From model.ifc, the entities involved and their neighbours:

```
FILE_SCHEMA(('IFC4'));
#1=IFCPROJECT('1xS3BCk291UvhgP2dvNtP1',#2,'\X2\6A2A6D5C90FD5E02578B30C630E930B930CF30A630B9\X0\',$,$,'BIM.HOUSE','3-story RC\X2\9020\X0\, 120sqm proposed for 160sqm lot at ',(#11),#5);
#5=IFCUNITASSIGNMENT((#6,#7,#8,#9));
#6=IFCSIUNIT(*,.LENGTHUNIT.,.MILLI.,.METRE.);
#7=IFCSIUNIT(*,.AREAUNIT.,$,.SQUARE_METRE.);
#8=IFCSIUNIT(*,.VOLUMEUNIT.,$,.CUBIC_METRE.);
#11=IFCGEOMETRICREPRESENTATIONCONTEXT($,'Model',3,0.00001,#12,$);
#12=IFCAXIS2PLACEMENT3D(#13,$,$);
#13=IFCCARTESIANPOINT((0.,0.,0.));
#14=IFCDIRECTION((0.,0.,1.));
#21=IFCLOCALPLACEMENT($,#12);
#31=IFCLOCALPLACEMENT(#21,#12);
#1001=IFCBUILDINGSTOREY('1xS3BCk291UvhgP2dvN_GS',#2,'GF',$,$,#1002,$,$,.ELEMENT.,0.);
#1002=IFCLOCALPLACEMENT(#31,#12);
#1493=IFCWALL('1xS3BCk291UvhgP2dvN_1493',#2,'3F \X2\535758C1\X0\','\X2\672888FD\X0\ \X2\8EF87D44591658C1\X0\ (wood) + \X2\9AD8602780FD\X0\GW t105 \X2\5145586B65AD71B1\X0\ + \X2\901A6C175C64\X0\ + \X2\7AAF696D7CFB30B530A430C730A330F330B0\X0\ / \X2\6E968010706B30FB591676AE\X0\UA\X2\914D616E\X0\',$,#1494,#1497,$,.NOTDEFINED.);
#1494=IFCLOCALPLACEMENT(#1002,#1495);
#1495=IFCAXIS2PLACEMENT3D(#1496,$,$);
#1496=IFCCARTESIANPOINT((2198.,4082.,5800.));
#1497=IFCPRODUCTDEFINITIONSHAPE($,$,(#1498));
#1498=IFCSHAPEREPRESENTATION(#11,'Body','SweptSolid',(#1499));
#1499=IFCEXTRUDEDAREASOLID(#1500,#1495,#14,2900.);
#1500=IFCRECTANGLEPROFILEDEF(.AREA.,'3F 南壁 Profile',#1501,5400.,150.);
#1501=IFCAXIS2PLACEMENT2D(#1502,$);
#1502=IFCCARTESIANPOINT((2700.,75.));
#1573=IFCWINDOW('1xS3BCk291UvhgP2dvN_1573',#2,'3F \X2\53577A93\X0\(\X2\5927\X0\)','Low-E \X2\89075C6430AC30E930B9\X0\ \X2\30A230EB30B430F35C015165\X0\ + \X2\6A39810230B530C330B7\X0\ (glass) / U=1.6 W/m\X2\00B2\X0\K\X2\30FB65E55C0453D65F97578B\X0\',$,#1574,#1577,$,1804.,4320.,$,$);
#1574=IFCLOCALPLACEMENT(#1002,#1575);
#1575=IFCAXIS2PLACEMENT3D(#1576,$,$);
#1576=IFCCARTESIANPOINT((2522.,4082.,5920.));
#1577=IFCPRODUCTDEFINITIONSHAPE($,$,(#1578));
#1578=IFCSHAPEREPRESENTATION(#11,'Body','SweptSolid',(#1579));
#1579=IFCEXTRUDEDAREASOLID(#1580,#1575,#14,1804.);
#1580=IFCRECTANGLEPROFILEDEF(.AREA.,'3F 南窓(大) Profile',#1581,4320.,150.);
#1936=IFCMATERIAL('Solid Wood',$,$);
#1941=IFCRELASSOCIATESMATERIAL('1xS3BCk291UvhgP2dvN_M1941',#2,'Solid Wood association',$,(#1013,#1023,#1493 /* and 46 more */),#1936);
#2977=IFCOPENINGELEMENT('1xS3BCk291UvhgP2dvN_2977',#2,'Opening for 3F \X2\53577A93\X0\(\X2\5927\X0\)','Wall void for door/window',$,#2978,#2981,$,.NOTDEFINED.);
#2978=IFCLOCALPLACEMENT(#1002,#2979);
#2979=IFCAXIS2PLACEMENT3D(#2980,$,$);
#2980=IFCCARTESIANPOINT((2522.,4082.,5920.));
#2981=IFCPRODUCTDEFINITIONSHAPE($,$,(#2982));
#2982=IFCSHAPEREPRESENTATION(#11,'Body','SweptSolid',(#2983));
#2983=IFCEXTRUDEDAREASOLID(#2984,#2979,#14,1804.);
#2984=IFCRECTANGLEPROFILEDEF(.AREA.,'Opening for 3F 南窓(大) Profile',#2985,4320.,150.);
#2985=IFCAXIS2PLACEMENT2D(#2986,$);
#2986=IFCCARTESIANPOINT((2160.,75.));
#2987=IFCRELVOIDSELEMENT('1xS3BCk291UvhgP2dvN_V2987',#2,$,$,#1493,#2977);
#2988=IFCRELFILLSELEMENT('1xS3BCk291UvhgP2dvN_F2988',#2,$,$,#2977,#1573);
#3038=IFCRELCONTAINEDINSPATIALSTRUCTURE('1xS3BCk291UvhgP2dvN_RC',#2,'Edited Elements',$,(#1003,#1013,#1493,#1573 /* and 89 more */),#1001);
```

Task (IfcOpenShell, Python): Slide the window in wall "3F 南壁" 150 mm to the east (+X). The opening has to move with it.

```python
import ifcopenshell
import ifcopenshell.api.geometry
import ifcopenshell.util.placement
import ifcopenshell.util.unit

model = ifcopenshell.open("model.ifc")
unit_scale = ifcopenshell.util.unit.calculate_unit_scale(model)

window = model.by_guid("1xS3BCk291UvhgP2dvN_1573")
opening = window.FillsVoids[0].RelatingOpeningElement
wall = opening.VoidsElements[0].RelatingBuildingElement

wall_matrix = ifcopenshell.util.placement.get_local_placement(wall.ObjectPlacement)
shift = wall_matrix[:3, 0] * 0.15 / unit_scale
before = ifcopenshell.util.placement.get_local_placement(window.ObjectPlacement)[:3, 3].copy()

# The window is not placed relative to its opening, so move both.
for product in (opening, window):
    matrix = ifcopenshell.util.placement.get_local_placement(product.ObjectPlacement)
    matrix[:3, 3] += shift
    ifcopenshell.api.geometry.edit_object_placement(model, product=product, matrix=matrix, is_si=False)

after = ifcopenshell.util.placement.get_local_placement(window.ObjectPlacement)[:3, 3]
print("window moved by", (after - before).round(3) + 0.0)

model.write("model_edited.ifc")
```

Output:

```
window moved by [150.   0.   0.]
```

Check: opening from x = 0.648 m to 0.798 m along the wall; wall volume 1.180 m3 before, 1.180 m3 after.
